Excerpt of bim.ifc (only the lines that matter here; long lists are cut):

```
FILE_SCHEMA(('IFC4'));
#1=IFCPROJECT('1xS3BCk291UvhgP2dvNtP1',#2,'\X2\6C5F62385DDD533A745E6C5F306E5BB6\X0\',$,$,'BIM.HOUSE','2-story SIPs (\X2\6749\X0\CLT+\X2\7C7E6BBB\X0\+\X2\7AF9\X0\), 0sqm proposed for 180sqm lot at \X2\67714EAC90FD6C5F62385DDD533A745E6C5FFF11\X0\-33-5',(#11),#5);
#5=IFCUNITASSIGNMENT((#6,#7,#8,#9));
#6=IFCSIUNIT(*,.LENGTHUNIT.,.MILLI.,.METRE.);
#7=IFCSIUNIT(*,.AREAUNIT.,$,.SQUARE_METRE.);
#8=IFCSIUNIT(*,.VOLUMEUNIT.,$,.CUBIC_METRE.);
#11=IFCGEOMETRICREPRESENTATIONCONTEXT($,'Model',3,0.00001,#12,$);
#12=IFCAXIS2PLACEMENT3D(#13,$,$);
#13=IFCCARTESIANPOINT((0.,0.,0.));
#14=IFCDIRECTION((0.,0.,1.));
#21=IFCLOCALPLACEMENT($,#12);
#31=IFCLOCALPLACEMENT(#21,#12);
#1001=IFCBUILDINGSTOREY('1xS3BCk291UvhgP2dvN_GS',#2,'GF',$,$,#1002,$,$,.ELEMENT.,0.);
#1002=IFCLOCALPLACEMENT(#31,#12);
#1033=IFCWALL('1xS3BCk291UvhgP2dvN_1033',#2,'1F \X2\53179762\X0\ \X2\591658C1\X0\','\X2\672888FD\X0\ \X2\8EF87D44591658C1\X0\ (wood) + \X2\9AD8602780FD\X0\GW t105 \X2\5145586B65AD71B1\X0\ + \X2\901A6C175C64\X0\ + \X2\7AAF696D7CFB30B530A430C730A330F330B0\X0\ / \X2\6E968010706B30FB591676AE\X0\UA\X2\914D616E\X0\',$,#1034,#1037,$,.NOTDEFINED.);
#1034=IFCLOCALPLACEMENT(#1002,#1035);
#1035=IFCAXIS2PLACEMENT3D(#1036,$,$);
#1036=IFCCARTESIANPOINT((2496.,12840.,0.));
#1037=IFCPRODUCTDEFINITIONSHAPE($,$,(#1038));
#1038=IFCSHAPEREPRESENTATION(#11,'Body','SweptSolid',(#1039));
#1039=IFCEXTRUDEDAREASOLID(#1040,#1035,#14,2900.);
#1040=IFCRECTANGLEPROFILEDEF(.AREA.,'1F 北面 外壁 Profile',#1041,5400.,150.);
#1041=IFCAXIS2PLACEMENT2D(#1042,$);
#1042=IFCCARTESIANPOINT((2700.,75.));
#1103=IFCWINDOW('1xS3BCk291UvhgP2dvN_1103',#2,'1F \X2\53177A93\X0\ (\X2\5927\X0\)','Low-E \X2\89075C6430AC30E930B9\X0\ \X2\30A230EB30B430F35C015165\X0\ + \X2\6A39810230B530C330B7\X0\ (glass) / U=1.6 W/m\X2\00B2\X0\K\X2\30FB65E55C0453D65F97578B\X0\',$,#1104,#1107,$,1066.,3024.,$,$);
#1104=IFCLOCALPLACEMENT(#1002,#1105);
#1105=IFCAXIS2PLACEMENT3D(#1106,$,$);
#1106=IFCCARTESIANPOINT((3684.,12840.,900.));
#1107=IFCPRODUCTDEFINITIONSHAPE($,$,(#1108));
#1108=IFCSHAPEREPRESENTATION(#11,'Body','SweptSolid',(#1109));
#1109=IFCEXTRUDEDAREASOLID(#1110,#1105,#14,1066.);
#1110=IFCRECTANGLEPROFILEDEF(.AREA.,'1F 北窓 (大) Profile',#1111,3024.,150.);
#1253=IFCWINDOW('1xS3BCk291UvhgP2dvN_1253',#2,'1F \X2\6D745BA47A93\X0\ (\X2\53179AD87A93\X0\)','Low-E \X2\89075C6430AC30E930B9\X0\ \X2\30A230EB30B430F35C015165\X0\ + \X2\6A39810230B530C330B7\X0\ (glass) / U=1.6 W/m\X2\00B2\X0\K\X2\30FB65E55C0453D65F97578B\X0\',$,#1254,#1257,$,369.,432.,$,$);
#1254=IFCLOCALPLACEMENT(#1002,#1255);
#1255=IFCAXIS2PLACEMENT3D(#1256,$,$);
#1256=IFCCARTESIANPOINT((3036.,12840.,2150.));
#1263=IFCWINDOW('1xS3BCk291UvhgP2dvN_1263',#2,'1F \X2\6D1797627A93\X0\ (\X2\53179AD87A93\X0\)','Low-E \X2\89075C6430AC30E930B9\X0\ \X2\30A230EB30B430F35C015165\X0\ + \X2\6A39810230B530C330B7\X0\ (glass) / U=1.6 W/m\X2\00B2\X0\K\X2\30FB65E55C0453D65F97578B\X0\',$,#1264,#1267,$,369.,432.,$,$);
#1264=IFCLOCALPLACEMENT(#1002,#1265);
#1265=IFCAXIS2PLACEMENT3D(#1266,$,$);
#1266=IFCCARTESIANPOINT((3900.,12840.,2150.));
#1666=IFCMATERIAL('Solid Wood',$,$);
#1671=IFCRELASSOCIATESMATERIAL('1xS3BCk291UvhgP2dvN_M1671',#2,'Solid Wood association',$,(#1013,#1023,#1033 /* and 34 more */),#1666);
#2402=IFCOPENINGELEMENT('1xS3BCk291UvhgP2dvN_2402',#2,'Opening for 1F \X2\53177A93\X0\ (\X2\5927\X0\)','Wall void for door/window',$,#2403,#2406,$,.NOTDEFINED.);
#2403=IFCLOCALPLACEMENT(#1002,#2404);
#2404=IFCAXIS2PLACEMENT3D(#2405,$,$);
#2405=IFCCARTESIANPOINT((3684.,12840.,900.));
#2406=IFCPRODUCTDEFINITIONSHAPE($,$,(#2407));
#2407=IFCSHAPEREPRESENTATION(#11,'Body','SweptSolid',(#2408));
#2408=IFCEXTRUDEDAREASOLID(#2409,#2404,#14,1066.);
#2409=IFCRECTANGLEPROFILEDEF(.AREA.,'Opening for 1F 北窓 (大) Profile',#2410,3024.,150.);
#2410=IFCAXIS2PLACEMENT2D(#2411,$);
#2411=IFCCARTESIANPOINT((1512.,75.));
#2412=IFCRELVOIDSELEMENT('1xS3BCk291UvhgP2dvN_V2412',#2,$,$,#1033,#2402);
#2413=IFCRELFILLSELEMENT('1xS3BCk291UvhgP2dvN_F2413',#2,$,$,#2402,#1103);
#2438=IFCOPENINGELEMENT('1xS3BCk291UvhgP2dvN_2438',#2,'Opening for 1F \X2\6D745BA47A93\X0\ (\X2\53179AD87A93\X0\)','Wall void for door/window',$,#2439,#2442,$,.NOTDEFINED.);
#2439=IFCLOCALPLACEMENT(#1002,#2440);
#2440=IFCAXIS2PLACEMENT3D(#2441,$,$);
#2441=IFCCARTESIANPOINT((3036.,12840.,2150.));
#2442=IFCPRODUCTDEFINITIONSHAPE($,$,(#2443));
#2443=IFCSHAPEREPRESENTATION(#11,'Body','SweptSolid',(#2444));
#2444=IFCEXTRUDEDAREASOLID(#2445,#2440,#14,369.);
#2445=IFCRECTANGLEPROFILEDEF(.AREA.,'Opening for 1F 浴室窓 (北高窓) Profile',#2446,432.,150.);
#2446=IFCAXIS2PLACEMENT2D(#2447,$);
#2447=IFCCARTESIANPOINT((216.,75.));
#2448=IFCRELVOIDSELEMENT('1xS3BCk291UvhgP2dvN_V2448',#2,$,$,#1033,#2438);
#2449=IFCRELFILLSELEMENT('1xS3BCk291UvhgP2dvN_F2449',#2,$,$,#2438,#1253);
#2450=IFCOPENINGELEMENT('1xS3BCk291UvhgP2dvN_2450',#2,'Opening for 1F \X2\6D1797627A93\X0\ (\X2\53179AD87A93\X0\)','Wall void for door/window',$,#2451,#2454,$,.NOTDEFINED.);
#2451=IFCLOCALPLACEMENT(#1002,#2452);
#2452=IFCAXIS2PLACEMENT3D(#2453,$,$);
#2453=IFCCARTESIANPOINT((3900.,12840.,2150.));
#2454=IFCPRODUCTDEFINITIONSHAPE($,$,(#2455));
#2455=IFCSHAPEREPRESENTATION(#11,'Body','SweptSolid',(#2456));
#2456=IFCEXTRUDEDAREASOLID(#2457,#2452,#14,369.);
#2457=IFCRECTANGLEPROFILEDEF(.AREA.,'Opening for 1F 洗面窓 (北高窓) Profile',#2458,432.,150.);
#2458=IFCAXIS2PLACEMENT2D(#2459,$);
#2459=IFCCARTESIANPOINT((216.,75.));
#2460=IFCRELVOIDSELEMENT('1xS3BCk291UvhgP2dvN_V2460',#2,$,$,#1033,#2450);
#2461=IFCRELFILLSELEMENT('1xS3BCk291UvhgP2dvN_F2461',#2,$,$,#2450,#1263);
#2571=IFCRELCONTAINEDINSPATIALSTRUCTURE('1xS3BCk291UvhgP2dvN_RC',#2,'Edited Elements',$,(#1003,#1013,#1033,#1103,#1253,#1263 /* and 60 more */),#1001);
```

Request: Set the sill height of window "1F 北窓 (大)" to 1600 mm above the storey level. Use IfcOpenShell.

```python
import numpy as np
import ifcopenshell
import ifcopenshell.api.geometry
import ifcopenshell.geom
import ifcopenshell.util.element
import ifcopenshell.util.placement
import ifcopenshell.util.shape
import ifcopenshell.util.unit

model = ifcopenshell.open("bim.ifc")
unit_scale = ifcopenshell.util.unit.calculate_unit_scale(model)

window = model.by_id(1103)
opening = window.FillsVoids[0].RelatingOpeningElement
storey = ifcopenshell.util.element.get_container(window, ifc_class="IfcBuildingStorey")
level = ifcopenshell.util.placement.get_local_placement(storey.ObjectPlacement)[2, 3]

# The opening's origin need not be at the sill, so measure its lowest point.
shape = ifcopenshell.geom.create_shape(ifcopenshell.geom.settings(), opening)
bottom = ifcopenshell.util.shape.get_shape_bottom_elevation(shape, shape.geometry) / unit_scale
dz = level + 1.6 / unit_scale - bottom

shift = np.array([0.0, 0.0, dz])
# The window is not placed relative to its opening, so move both.
for product in (opening, window):
    matrix = ifcopenshell.util.placement.get_local_placement(product.ObjectPlacement)
    matrix[:3, 3] += shift
    ifcopenshell.api.geometry.edit_object_placement(model, product=product, matrix=matrix, is_si=False)

print(f"moved by {dz * unit_scale:+.3f} m")

model.write("bim_edited.ifc")
```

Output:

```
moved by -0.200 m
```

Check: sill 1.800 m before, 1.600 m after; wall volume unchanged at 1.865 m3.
